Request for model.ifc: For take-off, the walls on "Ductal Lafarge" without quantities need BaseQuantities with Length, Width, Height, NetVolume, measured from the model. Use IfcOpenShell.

First a look at what the model holds.

```python
import ifcopenshell
import ifcopenshell.util.element
import ifcopenshell.util.unit

model = ifcopenshell.open("model.ifc")
print(model.schema)
for unit_type in ("LENGTHUNIT", "AREAUNIT", "VOLUMEUNIT"):
    print(unit_type, ifcopenshell.util.unit.calculate_unit_scale(model, unit_type))
storey = next(s for s in model.by_type("IfcBuildingStorey") if s.Name == "Ductal Lafarge")
walls = [e for e in ifcopenshell.util.element.get_decomposition(storey) if e.is_a("IfcWall")]
for e in sorted(walls, key=lambda e: e.id()):
    print(e.id(), e.is_a(), e.Name, list(ifcopenshell.util.element.get_psets(e, qtos_only=True)), sep=" | ")
```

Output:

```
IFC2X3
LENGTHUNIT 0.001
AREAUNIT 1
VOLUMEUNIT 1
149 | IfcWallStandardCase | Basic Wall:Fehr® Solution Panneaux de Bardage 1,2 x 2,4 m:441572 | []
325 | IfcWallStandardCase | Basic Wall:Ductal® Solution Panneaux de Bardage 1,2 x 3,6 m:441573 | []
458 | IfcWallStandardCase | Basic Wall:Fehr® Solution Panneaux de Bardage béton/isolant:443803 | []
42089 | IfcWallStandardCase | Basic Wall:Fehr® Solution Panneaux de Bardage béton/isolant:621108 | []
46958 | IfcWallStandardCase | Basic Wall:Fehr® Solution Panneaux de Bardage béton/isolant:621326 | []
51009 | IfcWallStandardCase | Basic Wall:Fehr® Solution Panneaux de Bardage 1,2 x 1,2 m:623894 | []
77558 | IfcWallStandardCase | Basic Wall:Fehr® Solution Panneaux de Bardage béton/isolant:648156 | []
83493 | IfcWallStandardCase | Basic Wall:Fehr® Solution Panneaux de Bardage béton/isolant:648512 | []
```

```python
import ifcopenshell
import ifcopenshell.api.pset
import ifcopenshell.geom
import ifcopenshell.util.element
import ifcopenshell.util.shape
import ifcopenshell.util.unit

model = ifcopenshell.open("model.ifc")
unit_scale = ifcopenshell.util.unit.calculate_unit_scale(model)
volume_scale = ifcopenshell.util.unit.calculate_unit_scale(model, "VOLUMEUNIT")
settings = ifcopenshell.geom.settings()

storey = next(s for s in model.by_type("IfcBuildingStorey") if s.Name == "Ductal Lafarge")
walls = [e for e in ifcopenshell.util.element.get_decomposition(storey) if e.is_a("IfcWall")]

for e in sorted(walls, key=lambda e: e.id()):
    if ifcopenshell.util.element.get_psets(e, qtos_only=True, should_inherit=False):
        continue
    # Geometry comes back in metres, in the element's own axes.
    shape = ifcopenshell.geom.create_shape(settings, e)
    values = {
        "Length": ifcopenshell.util.shape.get_x(shape.geometry) / unit_scale,
        "Width": ifcopenshell.util.shape.get_y(shape.geometry) / unit_scale,
        "Height": ifcopenshell.util.shape.get_z(shape.geometry) / unit_scale,
        "NetVolume": ifcopenshell.util.shape.get_volume(shape.geometry) / volume_scale,
    }
    qto = ifcopenshell.api.pset.add_qto(model, product=e, name="BaseQuantities")
    ifcopenshell.api.pset.edit_qto(model, qto=qto, properties=values)
    print(e.id(), {k: round(v, 3) for k, v in values.items()})

model.write("model_edited.ifc")
```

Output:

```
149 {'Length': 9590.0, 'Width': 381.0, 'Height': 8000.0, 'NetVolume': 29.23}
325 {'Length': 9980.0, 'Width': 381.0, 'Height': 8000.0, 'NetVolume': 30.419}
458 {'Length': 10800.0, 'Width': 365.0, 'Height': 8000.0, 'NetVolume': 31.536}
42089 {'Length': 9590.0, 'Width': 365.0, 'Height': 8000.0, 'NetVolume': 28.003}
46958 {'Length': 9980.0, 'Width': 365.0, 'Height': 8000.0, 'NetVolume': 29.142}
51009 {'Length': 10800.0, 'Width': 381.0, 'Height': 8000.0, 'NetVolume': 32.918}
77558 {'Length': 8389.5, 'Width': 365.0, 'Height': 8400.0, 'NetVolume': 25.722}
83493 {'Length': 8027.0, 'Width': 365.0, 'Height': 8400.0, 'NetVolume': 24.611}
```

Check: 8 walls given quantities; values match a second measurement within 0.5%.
